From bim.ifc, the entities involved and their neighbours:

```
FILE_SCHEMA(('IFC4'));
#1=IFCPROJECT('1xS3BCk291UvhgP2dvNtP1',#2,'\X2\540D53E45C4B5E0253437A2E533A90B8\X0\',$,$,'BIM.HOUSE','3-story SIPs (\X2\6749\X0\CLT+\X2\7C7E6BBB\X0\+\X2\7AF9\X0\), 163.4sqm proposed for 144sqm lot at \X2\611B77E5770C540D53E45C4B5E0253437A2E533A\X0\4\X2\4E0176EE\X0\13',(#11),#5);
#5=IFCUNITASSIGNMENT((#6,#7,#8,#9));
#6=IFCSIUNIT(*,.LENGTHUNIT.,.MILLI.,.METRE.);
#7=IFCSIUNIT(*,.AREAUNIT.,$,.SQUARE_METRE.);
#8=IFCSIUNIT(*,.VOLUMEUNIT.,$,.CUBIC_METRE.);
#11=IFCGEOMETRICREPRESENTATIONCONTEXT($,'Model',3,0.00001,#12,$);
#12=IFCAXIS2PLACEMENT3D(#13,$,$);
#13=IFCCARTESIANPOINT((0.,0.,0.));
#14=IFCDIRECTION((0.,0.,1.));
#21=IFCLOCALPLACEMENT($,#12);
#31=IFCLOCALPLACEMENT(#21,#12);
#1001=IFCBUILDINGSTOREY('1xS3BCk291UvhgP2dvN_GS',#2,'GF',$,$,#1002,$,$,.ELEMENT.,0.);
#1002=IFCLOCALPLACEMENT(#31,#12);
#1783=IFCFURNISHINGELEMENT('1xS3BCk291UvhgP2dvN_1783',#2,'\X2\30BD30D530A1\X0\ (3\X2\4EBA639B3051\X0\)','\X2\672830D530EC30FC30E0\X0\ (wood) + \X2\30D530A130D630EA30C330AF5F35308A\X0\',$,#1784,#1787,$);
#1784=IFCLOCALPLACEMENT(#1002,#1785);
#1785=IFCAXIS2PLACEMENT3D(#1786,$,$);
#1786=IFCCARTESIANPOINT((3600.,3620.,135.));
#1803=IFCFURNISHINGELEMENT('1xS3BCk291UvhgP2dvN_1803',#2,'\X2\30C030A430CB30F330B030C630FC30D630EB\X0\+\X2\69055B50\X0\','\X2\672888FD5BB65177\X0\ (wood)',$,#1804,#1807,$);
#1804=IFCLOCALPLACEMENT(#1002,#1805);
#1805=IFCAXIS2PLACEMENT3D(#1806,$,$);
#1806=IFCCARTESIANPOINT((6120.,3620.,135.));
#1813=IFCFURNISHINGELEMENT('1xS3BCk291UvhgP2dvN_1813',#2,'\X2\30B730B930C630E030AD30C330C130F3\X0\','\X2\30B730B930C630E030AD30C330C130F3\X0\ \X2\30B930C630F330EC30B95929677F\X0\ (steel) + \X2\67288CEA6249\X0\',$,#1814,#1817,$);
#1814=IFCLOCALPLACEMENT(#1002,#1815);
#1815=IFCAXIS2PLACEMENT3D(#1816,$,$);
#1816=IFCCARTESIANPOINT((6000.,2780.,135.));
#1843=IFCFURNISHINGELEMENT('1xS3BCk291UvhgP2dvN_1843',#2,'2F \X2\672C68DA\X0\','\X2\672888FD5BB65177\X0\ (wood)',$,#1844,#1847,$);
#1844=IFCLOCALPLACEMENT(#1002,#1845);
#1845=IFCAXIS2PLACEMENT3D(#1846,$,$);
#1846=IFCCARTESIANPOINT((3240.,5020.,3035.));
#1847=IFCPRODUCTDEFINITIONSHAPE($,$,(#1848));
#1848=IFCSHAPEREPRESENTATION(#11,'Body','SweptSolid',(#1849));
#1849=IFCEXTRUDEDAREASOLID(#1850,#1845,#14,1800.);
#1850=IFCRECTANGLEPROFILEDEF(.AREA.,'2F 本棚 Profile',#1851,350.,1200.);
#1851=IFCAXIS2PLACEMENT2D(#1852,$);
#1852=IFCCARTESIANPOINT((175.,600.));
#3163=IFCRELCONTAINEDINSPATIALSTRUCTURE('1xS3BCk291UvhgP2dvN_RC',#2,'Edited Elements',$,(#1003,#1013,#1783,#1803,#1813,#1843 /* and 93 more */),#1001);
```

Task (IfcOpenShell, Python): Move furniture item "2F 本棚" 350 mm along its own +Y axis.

```python
import ifcopenshell
import ifcopenshell.api.geometry
import ifcopenshell.util.placement
import ifcopenshell.util.unit

model = ifcopenshell.open("bim.ifc")
unit_scale = ifcopenshell.util.unit.calculate_unit_scale(model)

item = model.by_id(1843)
matrix = ifcopenshell.util.placement.get_local_placement(item.ObjectPlacement)
matrix[:3, 3] += matrix[:3, 1] * 0.35 / unit_scale
ifcopenshell.api.geometry.edit_object_placement(model, product=item, matrix=matrix, is_si=False)

print(ifcopenshell.util.placement.get_local_placement(item.ObjectPlacement).round(3) + 0.0)

model.write("bim_updated.ifc")
```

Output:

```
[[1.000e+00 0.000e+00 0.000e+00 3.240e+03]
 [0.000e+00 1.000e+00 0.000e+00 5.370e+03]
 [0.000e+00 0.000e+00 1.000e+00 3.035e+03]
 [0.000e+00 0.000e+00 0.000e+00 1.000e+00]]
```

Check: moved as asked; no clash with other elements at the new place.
